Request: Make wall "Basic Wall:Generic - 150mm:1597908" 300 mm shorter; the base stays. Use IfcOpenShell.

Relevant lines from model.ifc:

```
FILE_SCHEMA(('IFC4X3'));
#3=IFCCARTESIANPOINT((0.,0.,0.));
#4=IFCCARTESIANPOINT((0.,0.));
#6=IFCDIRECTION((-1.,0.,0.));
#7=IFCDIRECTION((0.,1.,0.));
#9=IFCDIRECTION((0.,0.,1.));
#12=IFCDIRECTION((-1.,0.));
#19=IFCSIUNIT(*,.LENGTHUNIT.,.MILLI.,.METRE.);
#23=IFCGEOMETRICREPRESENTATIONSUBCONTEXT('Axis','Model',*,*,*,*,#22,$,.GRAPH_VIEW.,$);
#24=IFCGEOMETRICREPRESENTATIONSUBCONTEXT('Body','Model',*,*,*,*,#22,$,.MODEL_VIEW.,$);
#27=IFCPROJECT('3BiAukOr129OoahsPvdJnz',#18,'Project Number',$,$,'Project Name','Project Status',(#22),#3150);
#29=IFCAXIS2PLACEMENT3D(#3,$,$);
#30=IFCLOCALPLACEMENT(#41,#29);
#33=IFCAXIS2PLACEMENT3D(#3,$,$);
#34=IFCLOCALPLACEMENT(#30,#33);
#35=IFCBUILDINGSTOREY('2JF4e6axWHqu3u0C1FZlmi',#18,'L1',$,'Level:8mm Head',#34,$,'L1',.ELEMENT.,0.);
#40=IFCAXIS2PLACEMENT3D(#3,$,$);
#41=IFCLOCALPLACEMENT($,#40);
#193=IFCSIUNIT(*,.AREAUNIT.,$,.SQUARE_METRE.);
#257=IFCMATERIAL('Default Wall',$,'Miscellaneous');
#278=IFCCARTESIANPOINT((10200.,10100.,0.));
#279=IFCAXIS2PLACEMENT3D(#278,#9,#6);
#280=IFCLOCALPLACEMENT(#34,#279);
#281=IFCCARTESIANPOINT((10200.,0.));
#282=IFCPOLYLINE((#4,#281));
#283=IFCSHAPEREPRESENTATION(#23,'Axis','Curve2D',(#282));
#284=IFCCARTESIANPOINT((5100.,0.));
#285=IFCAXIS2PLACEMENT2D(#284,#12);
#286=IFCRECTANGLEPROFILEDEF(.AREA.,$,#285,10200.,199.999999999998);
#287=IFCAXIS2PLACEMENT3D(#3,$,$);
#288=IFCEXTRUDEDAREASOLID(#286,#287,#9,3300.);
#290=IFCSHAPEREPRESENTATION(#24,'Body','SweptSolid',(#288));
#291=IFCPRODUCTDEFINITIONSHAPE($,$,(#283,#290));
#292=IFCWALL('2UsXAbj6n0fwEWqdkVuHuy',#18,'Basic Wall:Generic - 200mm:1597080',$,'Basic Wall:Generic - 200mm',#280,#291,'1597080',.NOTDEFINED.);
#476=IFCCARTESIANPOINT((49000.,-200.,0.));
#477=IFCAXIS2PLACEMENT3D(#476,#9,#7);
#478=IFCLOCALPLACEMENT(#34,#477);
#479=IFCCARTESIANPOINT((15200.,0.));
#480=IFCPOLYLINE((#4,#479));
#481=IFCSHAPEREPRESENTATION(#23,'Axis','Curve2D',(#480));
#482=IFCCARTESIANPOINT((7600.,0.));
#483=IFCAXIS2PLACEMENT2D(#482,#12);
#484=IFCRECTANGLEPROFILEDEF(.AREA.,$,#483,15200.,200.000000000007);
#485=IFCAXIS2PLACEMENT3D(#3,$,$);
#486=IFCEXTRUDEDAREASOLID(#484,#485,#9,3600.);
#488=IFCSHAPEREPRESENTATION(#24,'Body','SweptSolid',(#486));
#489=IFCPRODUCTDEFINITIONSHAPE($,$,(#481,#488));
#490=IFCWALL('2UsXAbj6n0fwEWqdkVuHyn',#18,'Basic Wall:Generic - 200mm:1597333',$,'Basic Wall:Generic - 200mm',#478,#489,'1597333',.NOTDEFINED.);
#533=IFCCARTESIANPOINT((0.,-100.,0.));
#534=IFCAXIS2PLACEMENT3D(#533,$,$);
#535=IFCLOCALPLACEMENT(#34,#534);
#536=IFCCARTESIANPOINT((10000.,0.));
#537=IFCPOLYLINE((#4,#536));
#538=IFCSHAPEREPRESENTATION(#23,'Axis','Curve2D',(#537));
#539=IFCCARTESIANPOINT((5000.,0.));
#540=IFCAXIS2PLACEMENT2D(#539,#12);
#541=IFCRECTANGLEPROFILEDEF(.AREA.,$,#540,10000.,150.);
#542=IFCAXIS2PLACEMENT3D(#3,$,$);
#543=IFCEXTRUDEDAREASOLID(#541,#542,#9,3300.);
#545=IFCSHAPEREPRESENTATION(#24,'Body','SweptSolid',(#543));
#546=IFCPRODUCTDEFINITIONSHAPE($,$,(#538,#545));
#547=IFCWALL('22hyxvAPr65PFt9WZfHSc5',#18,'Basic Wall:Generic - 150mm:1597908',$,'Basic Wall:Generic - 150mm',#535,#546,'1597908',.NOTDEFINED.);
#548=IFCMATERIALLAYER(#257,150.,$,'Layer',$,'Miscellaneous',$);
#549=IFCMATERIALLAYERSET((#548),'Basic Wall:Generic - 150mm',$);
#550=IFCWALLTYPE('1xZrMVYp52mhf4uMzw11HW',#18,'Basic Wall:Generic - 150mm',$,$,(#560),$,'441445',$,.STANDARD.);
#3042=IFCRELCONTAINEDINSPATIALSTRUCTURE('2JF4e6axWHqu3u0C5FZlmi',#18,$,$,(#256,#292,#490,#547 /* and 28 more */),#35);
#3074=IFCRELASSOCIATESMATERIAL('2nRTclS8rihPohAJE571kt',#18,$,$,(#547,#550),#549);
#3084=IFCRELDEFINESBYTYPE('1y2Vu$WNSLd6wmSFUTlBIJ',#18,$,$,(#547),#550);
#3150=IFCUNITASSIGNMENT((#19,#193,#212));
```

```python
import ifcopenshell
import ifcopenshell.geom
import ifcopenshell.util.representation
import ifcopenshell.util.shape
import ifcopenshell.util.unit

model = ifcopenshell.open("model.ifc")
unit_scale = ifcopenshell.util.unit.calculate_unit_scale(model)
settings = ifcopenshell.geom.settings()


def volume(element):
    """Net volume in cubic metres, openings subtracted."""
    shape = ifcopenshell.geom.create_shape(settings, element)
    return ifcopenshell.util.shape.get_volume(shape.geometry)


wall = model.by_guid("22hyxvAPr65PFt9WZfHSc5")
before = volume(wall)

body = ifcopenshell.util.representation.get_representation(wall, "Model", "Body")
solid = body.Items[0]
old_height = solid.Depth
solid.Depth -= 0.3 / unit_scale
after = volume(wall)

print(f"height {old_height:g} -> {solid.Depth:g}, volume {before:.3f} -> {after:.3f} m3")

model.write("model_rev.ifc")
```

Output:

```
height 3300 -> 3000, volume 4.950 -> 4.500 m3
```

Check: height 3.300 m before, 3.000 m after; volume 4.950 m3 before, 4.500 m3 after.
